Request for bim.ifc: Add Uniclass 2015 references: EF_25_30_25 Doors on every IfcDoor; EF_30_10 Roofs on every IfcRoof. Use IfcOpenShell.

First a look at what the model holds.

```python
import ifcopenshell

model = ifcopenshell.open("bim.ifc")
print(model.schema)
print("classifications:", [c.Name for c in model.by_type("IfcClassification")])
for ifc_class in ("IfcDoor", "IfcRoof", "IfcStair", "IfcWall", "IfcWindow"):
    print(ifc_class, len(model.by_type(ifc_class)))
```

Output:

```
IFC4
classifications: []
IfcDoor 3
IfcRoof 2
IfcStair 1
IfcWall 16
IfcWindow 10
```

```python
import ifcopenshell
import ifcopenshell.api.classification

model = ifcopenshell.open("bim.ifc")

system = ifcopenshell.api.classification.add_classification(model, classification="Uniclass 2015")

codes = {
    "IfcDoor": ("EF_25_30_25", "Doors"),
    "IfcRoof": ("EF_30_10", "Roofs"),
}
for ifc_class, (code, name) in codes.items():
    products = model.by_type(ifc_class)
    ifcopenshell.api.classification.add_reference(
        model, products=products, classification=system, identification=code, name=name
    )
    print(code, len(products))

model.write("bim_edited.ifc")
```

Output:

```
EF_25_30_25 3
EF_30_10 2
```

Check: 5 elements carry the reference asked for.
